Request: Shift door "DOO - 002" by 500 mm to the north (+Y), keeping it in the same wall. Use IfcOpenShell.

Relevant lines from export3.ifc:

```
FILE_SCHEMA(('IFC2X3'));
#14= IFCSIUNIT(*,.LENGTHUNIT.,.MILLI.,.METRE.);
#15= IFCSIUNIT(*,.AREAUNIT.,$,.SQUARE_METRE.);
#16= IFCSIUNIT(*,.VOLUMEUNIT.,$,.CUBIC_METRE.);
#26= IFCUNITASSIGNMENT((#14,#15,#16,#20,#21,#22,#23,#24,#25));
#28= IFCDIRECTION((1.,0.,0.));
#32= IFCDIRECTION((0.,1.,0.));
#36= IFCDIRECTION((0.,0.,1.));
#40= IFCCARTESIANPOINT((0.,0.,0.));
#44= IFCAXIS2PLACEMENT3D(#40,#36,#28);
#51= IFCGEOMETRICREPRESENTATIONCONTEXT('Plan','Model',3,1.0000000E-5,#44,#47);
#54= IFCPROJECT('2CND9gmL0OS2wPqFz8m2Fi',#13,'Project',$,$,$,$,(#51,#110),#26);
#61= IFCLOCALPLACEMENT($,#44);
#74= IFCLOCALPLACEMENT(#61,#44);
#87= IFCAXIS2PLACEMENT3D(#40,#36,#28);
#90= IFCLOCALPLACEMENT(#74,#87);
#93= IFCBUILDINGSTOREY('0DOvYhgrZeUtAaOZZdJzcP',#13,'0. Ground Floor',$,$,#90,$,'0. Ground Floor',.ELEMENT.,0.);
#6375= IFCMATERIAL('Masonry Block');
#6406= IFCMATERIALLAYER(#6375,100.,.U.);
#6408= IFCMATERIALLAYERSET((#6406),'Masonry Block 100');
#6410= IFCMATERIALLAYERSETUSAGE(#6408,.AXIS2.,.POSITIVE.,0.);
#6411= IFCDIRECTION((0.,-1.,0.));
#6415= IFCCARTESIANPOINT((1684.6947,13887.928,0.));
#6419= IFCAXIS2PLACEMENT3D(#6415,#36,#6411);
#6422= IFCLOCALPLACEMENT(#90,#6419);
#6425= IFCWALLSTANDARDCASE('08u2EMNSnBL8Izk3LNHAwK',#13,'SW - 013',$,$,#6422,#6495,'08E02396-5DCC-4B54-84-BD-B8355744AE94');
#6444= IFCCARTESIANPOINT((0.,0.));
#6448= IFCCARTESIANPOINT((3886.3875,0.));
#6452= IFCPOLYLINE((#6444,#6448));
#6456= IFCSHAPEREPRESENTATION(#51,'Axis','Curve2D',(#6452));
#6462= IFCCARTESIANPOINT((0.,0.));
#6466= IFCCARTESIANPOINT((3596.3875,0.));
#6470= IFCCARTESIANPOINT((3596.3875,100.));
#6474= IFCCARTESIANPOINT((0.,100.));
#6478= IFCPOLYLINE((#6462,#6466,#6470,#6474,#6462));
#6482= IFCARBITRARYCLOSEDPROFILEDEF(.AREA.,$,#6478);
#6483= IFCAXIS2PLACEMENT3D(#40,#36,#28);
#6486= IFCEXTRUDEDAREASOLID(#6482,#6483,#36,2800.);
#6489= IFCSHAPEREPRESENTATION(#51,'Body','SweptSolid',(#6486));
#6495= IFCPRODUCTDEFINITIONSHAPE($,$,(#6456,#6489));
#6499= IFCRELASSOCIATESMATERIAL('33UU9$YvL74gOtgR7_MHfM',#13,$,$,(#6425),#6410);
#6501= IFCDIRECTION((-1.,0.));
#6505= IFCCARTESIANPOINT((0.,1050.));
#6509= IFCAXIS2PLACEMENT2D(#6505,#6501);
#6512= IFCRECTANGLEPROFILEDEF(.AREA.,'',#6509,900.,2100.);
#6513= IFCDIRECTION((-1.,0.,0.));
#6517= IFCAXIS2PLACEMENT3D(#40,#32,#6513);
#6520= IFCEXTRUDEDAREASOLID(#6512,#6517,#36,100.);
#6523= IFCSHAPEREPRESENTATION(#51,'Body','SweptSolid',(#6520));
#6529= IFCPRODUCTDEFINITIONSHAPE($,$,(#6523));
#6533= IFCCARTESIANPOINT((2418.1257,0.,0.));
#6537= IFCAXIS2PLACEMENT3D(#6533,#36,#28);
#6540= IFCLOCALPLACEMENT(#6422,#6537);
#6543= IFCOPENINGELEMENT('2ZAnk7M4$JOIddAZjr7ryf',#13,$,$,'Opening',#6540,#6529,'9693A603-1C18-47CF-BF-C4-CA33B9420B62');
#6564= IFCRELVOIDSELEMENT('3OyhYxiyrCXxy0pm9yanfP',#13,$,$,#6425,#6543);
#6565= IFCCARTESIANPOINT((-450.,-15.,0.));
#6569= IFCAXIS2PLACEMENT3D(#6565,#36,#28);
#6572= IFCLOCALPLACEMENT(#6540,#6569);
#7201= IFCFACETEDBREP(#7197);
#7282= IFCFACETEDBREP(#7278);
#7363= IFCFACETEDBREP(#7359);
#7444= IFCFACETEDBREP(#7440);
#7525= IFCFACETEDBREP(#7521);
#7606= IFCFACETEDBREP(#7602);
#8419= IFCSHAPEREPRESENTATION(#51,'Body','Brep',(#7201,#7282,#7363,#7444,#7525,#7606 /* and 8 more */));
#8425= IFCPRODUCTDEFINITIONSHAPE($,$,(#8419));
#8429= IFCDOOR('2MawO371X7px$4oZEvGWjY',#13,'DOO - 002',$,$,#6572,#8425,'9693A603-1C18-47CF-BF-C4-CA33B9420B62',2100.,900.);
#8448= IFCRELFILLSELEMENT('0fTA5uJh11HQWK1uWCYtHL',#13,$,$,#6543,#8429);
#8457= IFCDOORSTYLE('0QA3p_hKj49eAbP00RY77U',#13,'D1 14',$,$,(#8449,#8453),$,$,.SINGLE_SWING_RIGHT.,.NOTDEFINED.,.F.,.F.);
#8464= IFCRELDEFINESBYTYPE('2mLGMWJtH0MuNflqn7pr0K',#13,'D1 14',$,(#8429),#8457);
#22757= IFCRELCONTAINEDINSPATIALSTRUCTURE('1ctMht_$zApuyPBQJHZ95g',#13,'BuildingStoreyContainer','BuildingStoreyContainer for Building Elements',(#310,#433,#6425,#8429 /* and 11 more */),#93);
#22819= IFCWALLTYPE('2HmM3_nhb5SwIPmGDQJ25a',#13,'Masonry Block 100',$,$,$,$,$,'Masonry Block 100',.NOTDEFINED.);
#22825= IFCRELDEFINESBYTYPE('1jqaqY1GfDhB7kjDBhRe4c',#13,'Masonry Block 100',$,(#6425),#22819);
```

```python
import ifcopenshell
import ifcopenshell.api.geometry
import ifcopenshell.util.placement

model = ifcopenshell.open("export3.ifc")

door = model.by_guid("2MawO371X7px$4oZEvGWjY")
opening = door.FillsVoids[0].RelatingOpeningElement
wall = opening.VoidsElements[0].RelatingBuildingElement

wall_matrix = ifcopenshell.util.placement.get_local_placement(wall.ObjectPlacement)
shift = wall_matrix[:3, 0] * -500.0
before = ifcopenshell.util.placement.get_local_placement(door.ObjectPlacement)[:3, 3].copy()

# The door is placed relative to its opening, so it follows when the opening moves.
matrix = ifcopenshell.util.placement.get_local_placement(opening.ObjectPlacement)
matrix[:3, 3] += shift
ifcopenshell.api.geometry.edit_object_placement(
    model, product=opening, matrix=matrix, is_si=False, should_transform_children=True
)

after = ifcopenshell.util.placement.get_local_placement(door.ObjectPlacement)[:3, 3]
print("door moved by", (after - before).round(3) + 0.0)

model.write("export3_updated.ifc")
```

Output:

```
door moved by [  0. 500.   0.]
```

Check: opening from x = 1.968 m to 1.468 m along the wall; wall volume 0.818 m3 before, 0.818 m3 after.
